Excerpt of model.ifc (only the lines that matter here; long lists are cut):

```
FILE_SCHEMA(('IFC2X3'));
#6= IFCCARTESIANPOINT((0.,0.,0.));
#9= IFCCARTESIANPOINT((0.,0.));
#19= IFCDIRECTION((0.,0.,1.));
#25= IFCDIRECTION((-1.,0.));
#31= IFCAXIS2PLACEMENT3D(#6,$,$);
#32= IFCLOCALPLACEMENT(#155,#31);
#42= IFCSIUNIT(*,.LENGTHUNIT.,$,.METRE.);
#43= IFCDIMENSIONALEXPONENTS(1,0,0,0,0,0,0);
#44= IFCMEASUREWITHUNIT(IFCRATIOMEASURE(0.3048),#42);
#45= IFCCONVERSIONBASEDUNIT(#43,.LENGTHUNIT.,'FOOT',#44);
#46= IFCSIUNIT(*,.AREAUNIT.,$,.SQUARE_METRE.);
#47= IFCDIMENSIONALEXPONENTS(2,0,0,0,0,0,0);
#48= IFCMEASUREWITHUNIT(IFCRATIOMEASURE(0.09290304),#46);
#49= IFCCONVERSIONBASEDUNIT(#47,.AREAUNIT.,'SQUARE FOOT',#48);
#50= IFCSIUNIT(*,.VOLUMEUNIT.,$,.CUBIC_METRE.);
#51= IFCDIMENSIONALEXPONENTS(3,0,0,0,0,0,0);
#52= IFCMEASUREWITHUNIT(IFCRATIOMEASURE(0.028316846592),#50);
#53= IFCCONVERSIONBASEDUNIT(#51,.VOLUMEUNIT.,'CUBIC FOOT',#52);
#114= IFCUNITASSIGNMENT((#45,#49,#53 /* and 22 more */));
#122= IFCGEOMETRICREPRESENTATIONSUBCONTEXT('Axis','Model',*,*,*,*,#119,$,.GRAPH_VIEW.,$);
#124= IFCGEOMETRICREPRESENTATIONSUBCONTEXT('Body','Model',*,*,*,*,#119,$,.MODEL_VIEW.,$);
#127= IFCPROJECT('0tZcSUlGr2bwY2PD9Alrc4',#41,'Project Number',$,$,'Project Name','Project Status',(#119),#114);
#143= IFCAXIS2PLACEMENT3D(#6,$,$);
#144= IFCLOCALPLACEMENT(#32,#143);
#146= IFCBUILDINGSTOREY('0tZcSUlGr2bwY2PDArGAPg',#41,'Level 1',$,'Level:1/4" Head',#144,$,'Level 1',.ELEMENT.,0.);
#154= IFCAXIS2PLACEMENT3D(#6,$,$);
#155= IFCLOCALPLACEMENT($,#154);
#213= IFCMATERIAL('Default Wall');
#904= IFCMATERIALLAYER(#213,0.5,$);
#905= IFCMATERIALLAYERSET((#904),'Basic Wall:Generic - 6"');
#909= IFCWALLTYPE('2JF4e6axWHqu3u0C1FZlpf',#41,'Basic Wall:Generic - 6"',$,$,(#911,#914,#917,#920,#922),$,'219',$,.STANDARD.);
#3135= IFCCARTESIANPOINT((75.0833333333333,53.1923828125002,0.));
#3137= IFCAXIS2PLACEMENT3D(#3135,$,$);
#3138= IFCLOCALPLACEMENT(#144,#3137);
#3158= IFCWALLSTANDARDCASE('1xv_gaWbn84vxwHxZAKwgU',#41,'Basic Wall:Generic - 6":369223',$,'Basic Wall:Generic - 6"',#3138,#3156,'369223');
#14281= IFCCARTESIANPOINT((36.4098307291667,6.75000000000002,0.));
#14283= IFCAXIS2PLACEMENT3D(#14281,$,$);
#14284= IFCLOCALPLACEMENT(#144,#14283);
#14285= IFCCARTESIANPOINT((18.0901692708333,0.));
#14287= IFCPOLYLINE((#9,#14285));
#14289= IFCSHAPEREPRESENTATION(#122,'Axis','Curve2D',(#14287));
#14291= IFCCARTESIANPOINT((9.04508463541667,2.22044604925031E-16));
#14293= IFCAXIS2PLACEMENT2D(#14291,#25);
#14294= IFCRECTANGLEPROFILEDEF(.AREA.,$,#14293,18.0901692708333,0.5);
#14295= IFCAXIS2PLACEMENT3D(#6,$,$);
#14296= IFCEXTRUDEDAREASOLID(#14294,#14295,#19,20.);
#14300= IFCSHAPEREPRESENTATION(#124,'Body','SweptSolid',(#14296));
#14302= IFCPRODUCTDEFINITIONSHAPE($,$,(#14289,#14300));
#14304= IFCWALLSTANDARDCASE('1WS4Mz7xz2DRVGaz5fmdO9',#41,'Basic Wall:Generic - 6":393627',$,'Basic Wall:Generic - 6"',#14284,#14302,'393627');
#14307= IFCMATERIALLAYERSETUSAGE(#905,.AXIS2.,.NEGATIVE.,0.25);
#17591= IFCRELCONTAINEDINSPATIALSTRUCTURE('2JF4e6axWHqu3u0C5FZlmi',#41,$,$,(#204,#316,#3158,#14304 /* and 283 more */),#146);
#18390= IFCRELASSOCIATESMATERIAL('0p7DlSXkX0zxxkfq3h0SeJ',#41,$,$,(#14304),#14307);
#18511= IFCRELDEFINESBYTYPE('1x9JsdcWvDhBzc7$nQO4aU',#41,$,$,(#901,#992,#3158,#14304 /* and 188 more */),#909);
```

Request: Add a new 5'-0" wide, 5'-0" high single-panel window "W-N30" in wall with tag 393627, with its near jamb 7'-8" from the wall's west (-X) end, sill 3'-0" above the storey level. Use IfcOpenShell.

```python
import numpy as np
import ifcopenshell
import ifcopenshell.api.feature
import ifcopenshell.api.geometry
import ifcopenshell.api.root
import ifcopenshell.api.spatial
import ifcopenshell.api.type
import ifcopenshell.geom
import ifcopenshell.util.element
import ifcopenshell.util.placement
import ifcopenshell.util.representation
import ifcopenshell.util.shape
import ifcopenshell.util.unit

model = ifcopenshell.open("model.ifc")
unit_scale = ifcopenshell.util.unit.calculate_unit_scale(model)
settings = ifcopenshell.geom.settings()


def volume(element):
    """Net volume in cubic metres, openings subtracted."""
    shape = ifcopenshell.geom.create_shape(settings, element)
    return ifcopenshell.util.shape.get_volume(shape.geometry)


wall = model.by_guid("1WS4Mz7xz2DRVGaz5fmdO9")
storey = ifcopenshell.util.element.get_container(wall, ifc_class="IfcBuildingStorey")
context = ifcopenshell.util.representation.get_context(model, "Model", "Body", "MODEL_VIEW")
before = volume(wall)

width, height, from_end, sill = 1.524, 1.524, 2.3368, 0.9144  # metres

# The wall runs along its own X axis, and the end named is its -X end.
wall_shape = ifcopenshell.geom.create_shape(settings, wall)
x, y, z = ifcopenshell.util.shape.get_vertices(wall_shape.geometry).T
start = x.min() + from_end
face, thickness = float(y.min()), float(y.max() - y.min())
wall_matrix = ifcopenshell.util.placement.get_local_placement(wall.ObjectPlacement)
level = ifcopenshell.util.placement.get_local_placement(storey.ObjectPlacement)[2, 3]


def in_wall(x, y):
    """Placement at x, y metres in the wall's axes, at sill height."""
    matrix = wall_matrix.copy()
    matrix[:, 3] = wall_matrix @ np.array([x / unit_scale, y / unit_scale, 0.0, 1.0])
    matrix[2, 3] = level + sill / unit_scale
    return matrix


# Opening: a box that overshoots both wall faces by 50 mm.
opening = ifcopenshell.api.root.create_entity(model, ifc_class="IfcOpeningElement")
box = ifcopenshell.api.geometry.add_wall_representation(
    model, context=context, length=width, height=height, thickness=thickness + 0.1
)
ifcopenshell.api.geometry.assign_representation(model, product=opening, representation=box)
ifcopenshell.api.geometry.edit_object_placement(model, product=opening, matrix=in_wall(start, face - 0.05), is_si=False)
ifcopenshell.api.feature.add_feature(model, feature=opening, element=wall)

window = ifcopenshell.api.root.create_entity(model, ifc_class="IfcWindow", name="W-N30")
window.OverallWidth, window.OverallHeight = width / unit_scale, height / unit_scale
body = ifcopenshell.api.geometry.add_window_representation(
    model,
    context=context,
    overall_width=window.OverallWidth,
    overall_height=window.OverallHeight,
    partition_type="SINGLE_PANEL",
)
ifcopenshell.api.geometry.assign_representation(model, product=window, representation=body)
ifcopenshell.api.spatial.assign_container(model, products=[window], relating_structure=storey)
fills = ifcopenshell.api.feature.add_filling(model, opening=opening, element=window)
fills.OwnerHistory = window.OwnerHistory  # required in IFC2X3

# IFC2X3 keeps the operation on the window style.
style = ifcopenshell.api.root.create_entity(model, ifc_class="IfcWindowStyle", name="W-N30")
style.OperationType, style.ConstructionType = "SINGLE_PANEL", "NOTDEFINED"
style.ParameterTakesPrecedence = style.Sizeable = False
ifcopenshell.api.type.assign_type(model, related_objects=[window], relating_type=style)

# Centre the window in the wall's thickness.
ifcopenshell.api.geometry.edit_object_placement(model, product=window, matrix=in_wall(start, face), is_si=False)
window_shape = ifcopenshell.geom.create_shape(settings, window)
depth = ifcopenshell.util.shape.get_vertices(window_shape.geometry)[:, 1]
offset = face + thickness / 2 - (depth.min() + depth.max()) / 2
ifcopenshell.api.geometry.edit_object_placement(model, product=window, matrix=in_wall(start, offset), is_si=False)

after = volume(wall)

print(f"wall volume {before:.3f} -> {after:.3f} m3")

model.write("model-out.ifc")
```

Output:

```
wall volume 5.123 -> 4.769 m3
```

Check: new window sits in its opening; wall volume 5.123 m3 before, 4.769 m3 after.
